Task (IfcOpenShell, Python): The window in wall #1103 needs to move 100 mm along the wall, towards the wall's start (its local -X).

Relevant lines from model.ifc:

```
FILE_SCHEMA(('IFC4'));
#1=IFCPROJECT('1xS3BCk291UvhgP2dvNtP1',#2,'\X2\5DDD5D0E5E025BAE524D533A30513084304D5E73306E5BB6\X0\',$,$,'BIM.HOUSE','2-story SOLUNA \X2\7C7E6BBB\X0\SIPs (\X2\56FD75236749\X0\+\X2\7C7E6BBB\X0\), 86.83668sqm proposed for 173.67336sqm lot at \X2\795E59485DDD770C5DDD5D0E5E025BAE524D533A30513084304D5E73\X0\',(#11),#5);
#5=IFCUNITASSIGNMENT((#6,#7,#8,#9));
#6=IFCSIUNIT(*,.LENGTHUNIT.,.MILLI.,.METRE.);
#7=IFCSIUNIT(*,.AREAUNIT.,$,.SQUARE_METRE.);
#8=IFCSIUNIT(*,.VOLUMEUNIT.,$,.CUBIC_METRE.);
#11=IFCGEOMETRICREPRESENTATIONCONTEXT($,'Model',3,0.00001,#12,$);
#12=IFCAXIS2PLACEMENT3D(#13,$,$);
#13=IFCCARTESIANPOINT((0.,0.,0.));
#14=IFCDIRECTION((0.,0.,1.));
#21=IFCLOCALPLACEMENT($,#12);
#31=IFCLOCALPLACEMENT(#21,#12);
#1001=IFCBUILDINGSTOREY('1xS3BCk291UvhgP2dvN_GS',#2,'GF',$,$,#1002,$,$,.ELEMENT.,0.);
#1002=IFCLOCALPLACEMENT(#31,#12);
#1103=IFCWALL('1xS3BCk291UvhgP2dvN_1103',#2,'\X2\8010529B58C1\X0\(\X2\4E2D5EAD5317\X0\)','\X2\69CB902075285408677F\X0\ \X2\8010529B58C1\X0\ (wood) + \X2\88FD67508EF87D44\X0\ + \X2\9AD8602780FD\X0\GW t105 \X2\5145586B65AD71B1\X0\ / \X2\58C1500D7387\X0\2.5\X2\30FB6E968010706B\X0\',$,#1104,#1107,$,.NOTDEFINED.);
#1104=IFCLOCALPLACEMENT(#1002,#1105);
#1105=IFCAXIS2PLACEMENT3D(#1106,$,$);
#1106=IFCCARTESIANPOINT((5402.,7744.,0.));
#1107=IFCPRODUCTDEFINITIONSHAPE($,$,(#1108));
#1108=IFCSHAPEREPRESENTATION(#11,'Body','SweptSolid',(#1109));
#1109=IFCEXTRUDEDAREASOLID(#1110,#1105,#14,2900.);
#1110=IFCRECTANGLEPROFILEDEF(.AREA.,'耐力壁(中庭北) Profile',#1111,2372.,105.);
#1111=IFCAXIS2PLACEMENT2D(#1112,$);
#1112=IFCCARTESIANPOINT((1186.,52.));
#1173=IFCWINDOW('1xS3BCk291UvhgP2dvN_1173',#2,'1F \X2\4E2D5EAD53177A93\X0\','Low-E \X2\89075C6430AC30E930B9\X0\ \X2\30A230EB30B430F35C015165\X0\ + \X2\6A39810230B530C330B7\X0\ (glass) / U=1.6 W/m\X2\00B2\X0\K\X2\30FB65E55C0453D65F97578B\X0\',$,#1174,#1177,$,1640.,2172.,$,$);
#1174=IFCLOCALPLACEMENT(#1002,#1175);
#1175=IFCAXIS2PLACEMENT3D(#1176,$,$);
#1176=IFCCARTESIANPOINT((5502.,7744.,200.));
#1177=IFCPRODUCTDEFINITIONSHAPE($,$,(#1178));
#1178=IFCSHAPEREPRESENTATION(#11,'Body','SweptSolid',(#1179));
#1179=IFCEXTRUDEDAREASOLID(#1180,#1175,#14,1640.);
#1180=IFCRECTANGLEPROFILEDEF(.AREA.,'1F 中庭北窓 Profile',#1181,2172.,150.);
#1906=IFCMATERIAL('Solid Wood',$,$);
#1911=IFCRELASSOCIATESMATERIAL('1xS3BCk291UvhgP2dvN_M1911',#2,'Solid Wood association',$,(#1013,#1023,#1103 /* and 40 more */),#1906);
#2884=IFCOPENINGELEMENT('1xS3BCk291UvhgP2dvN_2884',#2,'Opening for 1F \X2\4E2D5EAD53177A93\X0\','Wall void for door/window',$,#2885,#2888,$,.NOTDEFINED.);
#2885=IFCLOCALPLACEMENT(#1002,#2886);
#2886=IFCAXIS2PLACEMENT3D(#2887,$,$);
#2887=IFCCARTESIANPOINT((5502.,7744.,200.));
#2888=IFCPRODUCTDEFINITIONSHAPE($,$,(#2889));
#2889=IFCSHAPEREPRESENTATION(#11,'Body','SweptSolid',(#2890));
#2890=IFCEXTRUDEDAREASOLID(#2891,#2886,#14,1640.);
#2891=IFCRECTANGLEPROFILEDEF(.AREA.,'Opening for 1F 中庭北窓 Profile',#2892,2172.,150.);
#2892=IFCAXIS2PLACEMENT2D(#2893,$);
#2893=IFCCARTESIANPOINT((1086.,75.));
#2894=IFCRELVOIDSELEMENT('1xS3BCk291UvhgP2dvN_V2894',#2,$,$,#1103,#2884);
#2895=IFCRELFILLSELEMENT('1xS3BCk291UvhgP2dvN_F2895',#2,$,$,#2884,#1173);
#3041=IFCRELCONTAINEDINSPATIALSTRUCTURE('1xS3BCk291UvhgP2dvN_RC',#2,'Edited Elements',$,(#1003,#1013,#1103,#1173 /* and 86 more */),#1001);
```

```python
import ifcopenshell
import ifcopenshell.api.geometry
import ifcopenshell.util.placement

model = ifcopenshell.open("model.ifc")

window = model.by_guid("1xS3BCk291UvhgP2dvN_1173")
opening = window.FillsVoids[0].RelatingOpeningElement
wall = opening.VoidsElements[0].RelatingBuildingElement

wall_matrix = ifcopenshell.util.placement.get_local_placement(wall.ObjectPlacement)
shift = wall_matrix[:3, 0] * -100.0
before = ifcopenshell.util.placement.get_local_placement(window.ObjectPlacement)[:3, 3].copy()

# The window is not placed relative to its opening, so move both.
for product in (opening, window):
    matrix = ifcopenshell.util.placement.get_local_placement(product.ObjectPlacement)
    matrix[:3, 3] += shift
    ifcopenshell.api.geometry.edit_object_placement(model, product=product, matrix=matrix, is_si=False)

after = ifcopenshell.util.placement.get_local_placement(window.ObjectPlacement)[:3, 3]
print("window moved by", (after - before).round(3) + 0.0)

model.write("model_updated.ifc")
```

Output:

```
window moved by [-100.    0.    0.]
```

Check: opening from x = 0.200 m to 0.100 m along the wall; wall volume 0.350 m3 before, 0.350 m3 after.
